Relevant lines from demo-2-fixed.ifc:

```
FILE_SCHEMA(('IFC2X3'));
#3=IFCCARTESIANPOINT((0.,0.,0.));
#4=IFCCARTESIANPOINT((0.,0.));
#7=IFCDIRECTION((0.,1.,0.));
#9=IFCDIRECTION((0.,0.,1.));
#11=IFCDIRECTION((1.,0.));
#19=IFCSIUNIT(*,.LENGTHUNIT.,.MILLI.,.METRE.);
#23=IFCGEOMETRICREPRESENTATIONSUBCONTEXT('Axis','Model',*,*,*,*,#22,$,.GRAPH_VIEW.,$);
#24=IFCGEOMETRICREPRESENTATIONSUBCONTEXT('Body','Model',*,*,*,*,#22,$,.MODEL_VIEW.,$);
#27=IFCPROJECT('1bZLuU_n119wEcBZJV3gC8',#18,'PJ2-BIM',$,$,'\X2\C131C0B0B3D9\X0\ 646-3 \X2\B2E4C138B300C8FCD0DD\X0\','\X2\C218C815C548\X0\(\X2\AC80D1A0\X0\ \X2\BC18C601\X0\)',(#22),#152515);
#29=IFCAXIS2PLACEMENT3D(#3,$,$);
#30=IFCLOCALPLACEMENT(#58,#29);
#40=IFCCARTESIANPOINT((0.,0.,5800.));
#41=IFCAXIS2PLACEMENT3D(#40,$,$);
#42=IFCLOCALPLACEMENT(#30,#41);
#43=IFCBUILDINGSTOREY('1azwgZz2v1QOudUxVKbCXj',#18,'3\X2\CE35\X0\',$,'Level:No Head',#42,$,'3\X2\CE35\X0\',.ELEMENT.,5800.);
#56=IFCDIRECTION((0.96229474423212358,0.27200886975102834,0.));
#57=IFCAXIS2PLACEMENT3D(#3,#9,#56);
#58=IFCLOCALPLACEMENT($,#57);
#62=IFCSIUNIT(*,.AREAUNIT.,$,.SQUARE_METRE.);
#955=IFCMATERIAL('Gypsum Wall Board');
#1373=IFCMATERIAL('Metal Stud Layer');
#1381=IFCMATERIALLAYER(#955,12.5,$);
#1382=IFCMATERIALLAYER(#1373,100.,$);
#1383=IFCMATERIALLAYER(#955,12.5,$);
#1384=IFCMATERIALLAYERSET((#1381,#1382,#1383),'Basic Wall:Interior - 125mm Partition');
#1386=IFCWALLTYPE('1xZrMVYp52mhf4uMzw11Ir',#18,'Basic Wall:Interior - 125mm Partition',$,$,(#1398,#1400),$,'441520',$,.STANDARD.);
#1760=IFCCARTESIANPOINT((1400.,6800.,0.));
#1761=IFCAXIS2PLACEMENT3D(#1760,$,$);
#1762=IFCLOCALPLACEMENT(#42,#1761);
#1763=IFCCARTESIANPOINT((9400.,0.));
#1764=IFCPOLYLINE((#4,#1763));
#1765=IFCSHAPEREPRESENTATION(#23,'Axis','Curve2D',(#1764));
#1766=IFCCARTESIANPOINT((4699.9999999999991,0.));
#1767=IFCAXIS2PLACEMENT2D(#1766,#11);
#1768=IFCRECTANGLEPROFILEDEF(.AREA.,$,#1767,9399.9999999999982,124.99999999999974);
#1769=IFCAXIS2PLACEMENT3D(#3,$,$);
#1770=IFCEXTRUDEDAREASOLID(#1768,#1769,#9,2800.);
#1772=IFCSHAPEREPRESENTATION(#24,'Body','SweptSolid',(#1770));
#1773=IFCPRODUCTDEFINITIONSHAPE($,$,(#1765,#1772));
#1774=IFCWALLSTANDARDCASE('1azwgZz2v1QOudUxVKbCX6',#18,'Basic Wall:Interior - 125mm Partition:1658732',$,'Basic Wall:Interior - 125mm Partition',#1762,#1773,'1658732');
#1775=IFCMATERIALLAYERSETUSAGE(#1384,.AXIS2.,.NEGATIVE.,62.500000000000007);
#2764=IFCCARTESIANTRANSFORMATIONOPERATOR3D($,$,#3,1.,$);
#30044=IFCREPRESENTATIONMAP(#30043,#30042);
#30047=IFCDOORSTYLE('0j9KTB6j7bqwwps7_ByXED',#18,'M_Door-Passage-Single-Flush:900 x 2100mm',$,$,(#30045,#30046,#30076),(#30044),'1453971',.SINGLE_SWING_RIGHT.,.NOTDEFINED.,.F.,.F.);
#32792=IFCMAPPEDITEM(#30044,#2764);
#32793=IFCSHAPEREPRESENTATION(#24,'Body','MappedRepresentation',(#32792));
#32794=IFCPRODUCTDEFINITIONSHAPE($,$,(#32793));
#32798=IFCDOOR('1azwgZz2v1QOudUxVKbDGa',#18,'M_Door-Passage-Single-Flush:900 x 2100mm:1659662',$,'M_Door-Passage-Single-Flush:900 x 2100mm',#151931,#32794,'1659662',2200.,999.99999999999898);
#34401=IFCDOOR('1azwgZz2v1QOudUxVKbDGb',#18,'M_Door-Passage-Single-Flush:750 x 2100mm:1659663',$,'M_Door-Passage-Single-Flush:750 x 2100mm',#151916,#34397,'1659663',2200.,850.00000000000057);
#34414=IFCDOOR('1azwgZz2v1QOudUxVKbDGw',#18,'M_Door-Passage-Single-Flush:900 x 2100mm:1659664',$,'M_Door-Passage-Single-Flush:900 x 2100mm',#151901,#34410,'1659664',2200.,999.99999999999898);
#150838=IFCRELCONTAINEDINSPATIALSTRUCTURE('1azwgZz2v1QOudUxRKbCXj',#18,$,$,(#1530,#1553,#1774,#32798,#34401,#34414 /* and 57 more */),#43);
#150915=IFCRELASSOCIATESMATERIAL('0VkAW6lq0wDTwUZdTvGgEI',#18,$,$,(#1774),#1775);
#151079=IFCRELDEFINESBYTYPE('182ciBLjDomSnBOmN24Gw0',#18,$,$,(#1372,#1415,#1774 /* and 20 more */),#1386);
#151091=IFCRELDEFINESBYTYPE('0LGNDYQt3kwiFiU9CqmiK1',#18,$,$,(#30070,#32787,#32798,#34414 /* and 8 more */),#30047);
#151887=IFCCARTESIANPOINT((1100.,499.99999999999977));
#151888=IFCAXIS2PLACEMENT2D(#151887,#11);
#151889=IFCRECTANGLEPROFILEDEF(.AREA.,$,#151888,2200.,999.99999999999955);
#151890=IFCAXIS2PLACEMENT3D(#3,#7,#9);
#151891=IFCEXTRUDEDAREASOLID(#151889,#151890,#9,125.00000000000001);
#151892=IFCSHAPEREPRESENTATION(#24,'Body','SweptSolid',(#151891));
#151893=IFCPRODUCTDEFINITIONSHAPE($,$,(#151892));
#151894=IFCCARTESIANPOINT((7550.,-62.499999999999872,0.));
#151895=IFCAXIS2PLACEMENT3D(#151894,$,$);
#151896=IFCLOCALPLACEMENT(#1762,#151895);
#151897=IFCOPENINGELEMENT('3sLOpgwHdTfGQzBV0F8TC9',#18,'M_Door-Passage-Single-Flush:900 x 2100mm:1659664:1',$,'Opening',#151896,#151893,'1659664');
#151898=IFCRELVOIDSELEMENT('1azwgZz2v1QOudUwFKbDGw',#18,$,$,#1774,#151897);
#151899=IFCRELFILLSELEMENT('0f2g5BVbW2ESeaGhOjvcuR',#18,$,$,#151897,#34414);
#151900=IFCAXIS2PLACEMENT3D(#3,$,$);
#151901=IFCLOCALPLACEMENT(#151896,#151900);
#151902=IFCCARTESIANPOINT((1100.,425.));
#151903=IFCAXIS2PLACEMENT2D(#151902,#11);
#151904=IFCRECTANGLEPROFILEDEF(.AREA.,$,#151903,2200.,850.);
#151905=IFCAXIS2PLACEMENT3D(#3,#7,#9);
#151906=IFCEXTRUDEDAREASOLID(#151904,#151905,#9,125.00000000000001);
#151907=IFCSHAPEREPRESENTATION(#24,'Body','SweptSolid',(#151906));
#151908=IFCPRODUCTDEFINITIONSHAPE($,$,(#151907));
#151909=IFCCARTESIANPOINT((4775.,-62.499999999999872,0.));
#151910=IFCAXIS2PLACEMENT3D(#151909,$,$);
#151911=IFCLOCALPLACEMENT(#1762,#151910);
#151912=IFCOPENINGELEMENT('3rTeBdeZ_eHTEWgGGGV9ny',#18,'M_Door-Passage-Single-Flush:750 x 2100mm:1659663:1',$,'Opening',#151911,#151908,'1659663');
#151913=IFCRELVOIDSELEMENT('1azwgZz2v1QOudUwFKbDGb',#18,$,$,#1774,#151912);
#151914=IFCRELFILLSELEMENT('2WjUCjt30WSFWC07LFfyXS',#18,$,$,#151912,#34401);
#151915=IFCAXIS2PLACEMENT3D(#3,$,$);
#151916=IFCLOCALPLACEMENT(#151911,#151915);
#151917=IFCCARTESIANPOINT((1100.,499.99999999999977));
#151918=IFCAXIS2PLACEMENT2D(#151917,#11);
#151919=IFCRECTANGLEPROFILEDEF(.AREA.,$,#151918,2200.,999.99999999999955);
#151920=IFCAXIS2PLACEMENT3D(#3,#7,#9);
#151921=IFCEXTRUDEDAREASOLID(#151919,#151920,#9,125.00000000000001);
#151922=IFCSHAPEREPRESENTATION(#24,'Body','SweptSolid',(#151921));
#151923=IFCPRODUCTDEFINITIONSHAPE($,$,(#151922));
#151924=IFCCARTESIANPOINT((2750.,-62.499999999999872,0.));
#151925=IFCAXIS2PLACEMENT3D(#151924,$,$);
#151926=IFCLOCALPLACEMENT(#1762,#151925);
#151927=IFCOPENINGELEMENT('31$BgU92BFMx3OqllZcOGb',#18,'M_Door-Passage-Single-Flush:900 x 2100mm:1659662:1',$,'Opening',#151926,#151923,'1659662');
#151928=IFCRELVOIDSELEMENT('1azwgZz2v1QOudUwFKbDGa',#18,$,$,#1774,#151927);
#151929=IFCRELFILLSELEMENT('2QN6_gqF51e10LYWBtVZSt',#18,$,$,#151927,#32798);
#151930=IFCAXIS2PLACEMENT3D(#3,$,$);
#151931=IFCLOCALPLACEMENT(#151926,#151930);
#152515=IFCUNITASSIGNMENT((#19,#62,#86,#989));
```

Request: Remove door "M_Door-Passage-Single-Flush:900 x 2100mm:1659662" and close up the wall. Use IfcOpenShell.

```python
import ifcopenshell
import ifcopenshell.api.feature
import ifcopenshell.api.root
import ifcopenshell.geom
import ifcopenshell.util.shape

model = ifcopenshell.open("demo-2-fixed.ifc")
settings = ifcopenshell.geom.settings()


def volume(element):
    """Net volume in cubic metres, openings subtracted."""
    shape = ifcopenshell.geom.create_shape(settings, element)
    return ifcopenshell.util.shape.get_volume(shape.geometry)


door = model.by_id(32798)
opening = door.FillsVoids[0].RelatingOpeningElement
wall = opening.VoidsElements[0].RelatingBuildingElement
before = volume(wall)

ifcopenshell.api.root.remove_product(model, product=door)
ifcopenshell.api.feature.remove_feature(model, feature=opening)

after = volume(wall)

print(f"wall volume {before:.3f} -> {after:.3f} m3")

model.write("demo-2-fixed_updated.ifc")
```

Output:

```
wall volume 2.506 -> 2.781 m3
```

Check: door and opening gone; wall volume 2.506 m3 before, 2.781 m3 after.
